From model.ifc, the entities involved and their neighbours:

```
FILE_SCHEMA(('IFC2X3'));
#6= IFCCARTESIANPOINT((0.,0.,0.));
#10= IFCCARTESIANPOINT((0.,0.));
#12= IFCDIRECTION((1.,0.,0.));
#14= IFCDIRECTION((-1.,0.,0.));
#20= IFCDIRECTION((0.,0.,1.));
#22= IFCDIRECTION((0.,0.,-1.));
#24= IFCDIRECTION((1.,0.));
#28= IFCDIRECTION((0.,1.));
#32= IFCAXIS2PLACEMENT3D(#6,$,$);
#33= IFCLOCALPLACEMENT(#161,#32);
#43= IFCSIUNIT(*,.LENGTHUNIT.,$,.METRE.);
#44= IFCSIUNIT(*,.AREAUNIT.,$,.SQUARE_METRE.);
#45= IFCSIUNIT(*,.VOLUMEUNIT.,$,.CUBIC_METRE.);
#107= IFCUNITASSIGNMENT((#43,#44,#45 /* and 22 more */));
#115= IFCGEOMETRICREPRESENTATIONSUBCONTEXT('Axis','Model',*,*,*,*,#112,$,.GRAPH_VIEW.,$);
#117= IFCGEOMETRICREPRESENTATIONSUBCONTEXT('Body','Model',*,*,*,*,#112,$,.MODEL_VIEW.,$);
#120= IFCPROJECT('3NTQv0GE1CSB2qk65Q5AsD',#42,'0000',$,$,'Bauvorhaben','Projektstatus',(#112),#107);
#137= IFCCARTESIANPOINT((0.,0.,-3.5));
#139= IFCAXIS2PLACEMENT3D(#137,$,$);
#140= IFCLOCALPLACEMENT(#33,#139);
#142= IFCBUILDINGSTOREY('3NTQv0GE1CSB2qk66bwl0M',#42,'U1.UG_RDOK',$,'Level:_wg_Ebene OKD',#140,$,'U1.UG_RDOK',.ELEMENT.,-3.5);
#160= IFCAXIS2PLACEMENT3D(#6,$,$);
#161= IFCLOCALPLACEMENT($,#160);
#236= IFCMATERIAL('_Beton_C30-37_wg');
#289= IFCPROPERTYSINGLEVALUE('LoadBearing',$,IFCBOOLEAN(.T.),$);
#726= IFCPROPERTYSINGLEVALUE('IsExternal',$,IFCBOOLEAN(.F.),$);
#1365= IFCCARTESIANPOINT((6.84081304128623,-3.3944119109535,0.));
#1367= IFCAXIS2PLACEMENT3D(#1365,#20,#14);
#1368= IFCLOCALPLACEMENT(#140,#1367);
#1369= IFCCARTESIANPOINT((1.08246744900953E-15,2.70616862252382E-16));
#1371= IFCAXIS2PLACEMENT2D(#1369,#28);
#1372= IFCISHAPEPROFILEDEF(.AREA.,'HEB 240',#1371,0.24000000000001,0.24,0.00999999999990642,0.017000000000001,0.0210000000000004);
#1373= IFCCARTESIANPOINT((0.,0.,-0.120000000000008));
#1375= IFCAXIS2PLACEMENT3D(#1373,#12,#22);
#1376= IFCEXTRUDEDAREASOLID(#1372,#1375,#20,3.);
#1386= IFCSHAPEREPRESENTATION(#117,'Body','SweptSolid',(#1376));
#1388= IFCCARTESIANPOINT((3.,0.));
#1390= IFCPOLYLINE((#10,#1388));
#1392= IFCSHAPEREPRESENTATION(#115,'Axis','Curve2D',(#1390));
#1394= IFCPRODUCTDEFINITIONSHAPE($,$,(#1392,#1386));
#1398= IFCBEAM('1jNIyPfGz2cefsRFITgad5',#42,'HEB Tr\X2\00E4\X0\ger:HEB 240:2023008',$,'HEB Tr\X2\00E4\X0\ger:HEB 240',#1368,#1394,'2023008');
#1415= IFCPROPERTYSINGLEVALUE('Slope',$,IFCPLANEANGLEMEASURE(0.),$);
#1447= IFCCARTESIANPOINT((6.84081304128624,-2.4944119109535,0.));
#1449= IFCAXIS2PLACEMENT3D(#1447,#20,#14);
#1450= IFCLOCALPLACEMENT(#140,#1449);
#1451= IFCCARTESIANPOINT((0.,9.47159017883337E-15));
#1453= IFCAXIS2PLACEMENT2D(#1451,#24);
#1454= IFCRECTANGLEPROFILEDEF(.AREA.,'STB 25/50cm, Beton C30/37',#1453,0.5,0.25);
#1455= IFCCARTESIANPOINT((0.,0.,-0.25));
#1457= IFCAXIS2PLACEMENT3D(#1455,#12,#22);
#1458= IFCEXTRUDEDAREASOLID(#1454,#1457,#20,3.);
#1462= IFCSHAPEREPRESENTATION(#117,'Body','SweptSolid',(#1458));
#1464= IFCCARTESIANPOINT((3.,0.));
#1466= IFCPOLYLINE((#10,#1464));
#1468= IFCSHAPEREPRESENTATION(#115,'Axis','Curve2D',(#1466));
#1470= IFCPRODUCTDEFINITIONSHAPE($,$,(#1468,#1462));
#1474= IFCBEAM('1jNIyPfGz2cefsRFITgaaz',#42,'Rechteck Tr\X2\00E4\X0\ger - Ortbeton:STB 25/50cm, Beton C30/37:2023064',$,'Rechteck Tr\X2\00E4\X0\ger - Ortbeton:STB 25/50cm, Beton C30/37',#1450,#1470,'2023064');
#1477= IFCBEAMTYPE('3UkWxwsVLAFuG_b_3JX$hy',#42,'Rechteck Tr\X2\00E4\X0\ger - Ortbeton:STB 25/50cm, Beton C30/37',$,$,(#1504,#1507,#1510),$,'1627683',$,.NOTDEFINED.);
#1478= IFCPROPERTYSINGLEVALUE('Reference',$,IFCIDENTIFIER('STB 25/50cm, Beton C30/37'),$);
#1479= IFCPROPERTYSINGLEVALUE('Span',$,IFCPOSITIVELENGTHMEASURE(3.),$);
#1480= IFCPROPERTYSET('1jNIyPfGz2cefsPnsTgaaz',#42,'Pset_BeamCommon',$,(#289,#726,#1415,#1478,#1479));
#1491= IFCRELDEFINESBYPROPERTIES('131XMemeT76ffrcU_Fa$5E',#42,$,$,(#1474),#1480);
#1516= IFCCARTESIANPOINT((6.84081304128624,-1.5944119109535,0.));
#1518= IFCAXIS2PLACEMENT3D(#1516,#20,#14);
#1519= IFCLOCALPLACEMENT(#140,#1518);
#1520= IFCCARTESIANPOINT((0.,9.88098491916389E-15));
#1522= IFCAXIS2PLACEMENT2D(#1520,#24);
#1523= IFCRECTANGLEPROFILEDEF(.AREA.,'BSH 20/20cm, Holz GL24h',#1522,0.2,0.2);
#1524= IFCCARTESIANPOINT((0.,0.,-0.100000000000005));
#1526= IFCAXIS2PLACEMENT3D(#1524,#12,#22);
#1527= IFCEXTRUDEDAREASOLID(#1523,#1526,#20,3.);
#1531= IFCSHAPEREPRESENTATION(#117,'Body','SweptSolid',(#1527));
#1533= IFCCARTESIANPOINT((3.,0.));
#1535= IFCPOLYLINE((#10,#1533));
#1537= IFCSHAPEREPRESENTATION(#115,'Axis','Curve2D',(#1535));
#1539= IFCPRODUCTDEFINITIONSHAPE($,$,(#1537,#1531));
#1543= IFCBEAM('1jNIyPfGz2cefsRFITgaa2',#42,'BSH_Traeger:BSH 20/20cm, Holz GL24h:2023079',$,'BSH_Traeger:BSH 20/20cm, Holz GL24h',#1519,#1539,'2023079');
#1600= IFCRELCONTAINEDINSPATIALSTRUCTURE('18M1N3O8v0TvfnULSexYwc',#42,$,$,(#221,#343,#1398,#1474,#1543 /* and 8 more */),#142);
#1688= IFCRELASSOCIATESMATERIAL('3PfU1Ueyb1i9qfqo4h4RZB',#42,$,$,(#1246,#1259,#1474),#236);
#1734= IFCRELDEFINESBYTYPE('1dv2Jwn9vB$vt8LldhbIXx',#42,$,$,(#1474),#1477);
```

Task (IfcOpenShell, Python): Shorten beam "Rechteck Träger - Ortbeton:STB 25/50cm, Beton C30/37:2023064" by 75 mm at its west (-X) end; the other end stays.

```python
import numpy as np
import ifcopenshell
import ifcopenshell.api.pset
import ifcopenshell.util.element
import ifcopenshell.util.representation

model = ifcopenshell.open("model.ifc")

member = model.by_guid("1jNIyPfGz2cefsRFITgaaz")
change = -0.075

# The extrusion runs towards the end named, so only its depth changes.
body = ifcopenshell.util.representation.get_representation(member, "Model", "Body")
solid = body.Items[0]
old_length = solid.Depth
solid.Depth += change

# Move the axis end point with it.
axis = next(r for r in member.Representation.Representations if r.RepresentationIdentifier == "Axis").Items[0]
start, end = (np.array(p.Coordinates) for p in axis.Points)
end = end + (end - start) / np.linalg.norm(end - start) * change
point = model.createIfcCartesianPoint(end.tolist())
axis.Points = [axis.Points[0], point]

# Update the stored length and volume.
pset = model.by_id(ifcopenshell.util.element.get_pset(member, "Pset_BeamCommon", should_inherit=False)["id"])
ifcopenshell.api.pset.edit_pset(model, pset=pset, properties={
    "Span": model.create_entity("IfcPositiveLengthMeasure", solid.Depth),
})

print(f"length {old_length:g} -> {solid.Depth:g}")

model.write("model_edited.ifc")
```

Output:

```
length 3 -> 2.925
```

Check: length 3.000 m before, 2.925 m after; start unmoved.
